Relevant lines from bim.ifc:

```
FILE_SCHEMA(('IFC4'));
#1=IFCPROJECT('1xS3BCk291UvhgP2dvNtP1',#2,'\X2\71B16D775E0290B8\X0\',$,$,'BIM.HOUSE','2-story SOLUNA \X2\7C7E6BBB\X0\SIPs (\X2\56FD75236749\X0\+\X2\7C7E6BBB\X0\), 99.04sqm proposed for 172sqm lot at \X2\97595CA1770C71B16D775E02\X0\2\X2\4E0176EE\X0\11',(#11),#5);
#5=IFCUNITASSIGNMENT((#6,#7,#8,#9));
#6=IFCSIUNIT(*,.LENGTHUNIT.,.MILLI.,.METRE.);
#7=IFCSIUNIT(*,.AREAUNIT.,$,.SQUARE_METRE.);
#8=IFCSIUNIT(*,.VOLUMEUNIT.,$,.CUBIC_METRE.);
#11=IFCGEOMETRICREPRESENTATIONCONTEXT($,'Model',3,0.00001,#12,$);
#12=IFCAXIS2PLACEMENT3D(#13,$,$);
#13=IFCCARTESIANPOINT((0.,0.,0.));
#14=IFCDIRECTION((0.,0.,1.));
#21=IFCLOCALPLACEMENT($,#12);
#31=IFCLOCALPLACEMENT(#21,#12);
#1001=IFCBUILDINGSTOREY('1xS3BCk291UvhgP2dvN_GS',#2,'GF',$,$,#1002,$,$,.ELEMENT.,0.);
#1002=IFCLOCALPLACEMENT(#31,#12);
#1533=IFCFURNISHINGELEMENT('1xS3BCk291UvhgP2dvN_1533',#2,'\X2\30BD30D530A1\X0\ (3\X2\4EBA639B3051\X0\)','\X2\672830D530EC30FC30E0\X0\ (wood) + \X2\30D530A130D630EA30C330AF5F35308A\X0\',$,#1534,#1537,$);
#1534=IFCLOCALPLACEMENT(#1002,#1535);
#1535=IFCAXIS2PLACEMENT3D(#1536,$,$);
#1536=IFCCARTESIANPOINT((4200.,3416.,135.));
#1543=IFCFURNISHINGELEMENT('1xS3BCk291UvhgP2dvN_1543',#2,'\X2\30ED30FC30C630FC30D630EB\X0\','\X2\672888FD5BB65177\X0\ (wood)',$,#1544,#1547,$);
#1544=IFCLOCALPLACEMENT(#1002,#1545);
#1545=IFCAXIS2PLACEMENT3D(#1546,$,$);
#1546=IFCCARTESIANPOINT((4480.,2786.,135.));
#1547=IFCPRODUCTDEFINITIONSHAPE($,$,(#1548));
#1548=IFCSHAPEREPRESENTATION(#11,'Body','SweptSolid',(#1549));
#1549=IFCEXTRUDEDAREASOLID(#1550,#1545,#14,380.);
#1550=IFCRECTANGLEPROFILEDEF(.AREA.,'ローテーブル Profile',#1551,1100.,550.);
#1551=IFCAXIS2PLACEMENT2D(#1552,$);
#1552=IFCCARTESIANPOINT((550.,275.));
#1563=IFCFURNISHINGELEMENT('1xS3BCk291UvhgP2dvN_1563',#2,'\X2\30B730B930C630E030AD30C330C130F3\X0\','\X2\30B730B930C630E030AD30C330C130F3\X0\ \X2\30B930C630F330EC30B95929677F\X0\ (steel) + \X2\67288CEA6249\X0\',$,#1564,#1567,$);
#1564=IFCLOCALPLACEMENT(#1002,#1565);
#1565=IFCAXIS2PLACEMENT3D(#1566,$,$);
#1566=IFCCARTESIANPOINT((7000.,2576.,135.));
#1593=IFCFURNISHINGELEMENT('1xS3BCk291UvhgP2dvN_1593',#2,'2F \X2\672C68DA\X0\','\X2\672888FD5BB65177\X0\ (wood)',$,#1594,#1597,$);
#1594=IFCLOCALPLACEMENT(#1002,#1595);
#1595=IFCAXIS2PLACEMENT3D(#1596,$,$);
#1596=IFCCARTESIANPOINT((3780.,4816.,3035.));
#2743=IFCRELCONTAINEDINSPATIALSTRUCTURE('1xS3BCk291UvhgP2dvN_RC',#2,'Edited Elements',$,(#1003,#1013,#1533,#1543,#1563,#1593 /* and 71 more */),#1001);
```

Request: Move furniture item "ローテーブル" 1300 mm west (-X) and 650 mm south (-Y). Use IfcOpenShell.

```python
import ifcopenshell
import ifcopenshell.api.geometry
import ifcopenshell.util.placement
import ifcopenshell.util.unit

model = ifcopenshell.open("bim.ifc")
unit_scale = ifcopenshell.util.unit.calculate_unit_scale(model)

item = model.by_guid("1xS3BCk291UvhgP2dvN_1543")
matrix = ifcopenshell.util.placement.get_local_placement(item.ObjectPlacement)
matrix[0, 3] -= 1.3 / unit_scale
matrix[1, 3] -= 0.65 / unit_scale
ifcopenshell.api.geometry.edit_object_placement(model, product=item, matrix=matrix, is_si=False)

print(ifcopenshell.util.placement.get_local_placement(item.ObjectPlacement).round(3) + 0.0)

model.write("bim_edited.ifc")
```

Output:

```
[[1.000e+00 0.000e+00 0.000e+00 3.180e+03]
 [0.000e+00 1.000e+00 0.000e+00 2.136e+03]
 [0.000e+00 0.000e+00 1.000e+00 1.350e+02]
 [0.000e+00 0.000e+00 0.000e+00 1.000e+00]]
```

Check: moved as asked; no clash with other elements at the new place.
